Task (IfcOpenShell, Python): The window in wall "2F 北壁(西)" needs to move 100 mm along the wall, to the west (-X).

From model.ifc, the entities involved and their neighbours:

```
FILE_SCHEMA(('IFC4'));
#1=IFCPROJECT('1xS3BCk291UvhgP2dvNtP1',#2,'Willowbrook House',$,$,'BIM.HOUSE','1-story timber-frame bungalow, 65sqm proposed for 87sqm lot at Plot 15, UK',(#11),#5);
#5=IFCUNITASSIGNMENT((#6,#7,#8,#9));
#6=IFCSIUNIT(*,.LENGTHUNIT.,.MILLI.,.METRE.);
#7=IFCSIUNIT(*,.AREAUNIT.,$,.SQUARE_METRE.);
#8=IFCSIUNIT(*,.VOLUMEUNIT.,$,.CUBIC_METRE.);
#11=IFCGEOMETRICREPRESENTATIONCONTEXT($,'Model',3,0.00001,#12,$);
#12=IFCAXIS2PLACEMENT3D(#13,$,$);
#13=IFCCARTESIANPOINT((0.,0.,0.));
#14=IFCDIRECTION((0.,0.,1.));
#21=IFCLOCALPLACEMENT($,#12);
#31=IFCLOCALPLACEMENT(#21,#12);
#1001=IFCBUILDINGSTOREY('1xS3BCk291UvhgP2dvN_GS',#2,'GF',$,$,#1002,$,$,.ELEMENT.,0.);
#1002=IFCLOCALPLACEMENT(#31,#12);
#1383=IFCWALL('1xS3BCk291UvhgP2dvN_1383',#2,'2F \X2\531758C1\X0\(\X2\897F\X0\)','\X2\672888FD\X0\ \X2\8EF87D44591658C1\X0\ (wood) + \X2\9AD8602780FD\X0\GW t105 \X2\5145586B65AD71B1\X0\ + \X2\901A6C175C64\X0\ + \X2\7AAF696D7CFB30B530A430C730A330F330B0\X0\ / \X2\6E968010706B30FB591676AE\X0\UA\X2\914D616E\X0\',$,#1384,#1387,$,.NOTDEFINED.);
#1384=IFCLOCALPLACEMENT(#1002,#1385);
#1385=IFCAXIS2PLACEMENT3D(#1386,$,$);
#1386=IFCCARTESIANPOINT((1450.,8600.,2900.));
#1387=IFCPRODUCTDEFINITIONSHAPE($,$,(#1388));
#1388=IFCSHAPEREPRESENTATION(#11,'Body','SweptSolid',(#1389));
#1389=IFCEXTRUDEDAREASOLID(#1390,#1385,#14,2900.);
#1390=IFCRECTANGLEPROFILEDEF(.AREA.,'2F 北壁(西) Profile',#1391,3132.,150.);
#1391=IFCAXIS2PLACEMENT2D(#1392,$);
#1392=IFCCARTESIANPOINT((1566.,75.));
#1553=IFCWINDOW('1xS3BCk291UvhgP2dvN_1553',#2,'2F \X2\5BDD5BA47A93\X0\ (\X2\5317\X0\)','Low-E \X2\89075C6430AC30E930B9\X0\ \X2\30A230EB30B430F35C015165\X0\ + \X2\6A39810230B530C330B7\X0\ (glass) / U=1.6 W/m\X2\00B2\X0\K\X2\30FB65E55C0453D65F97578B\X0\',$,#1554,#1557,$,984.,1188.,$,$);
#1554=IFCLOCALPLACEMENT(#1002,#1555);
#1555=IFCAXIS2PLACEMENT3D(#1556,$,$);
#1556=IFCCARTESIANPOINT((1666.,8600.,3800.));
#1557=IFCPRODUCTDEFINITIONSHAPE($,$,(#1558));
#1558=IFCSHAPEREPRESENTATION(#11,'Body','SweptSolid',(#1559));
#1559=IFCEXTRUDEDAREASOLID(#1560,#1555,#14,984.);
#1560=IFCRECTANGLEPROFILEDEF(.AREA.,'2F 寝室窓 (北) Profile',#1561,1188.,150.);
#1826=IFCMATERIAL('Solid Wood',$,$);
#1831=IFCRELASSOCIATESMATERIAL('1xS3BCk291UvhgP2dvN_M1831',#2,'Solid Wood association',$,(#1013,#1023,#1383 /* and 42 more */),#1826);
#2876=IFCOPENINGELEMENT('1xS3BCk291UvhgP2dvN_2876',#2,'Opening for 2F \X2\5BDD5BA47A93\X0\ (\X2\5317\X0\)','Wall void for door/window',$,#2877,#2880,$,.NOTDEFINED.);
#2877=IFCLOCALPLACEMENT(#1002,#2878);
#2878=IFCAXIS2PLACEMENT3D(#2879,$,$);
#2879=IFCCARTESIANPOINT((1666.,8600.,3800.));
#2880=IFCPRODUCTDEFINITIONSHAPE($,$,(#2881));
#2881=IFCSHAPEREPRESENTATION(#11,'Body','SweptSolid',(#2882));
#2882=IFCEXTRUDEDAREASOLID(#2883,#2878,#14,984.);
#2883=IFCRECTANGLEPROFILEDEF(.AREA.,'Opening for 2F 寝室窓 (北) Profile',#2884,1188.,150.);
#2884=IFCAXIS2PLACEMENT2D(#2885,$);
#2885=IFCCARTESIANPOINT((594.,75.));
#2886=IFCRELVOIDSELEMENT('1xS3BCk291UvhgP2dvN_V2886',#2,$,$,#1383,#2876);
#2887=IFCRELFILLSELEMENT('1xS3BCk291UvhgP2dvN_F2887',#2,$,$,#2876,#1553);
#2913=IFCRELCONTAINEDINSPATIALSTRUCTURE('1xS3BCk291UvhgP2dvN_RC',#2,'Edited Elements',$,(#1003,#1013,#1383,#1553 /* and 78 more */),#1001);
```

```python
import ifcopenshell
import ifcopenshell.api.geometry
import ifcopenshell.util.placement

model = ifcopenshell.open("model.ifc")

window = model.by_guid("1xS3BCk291UvhgP2dvN_1553")
opening = window.FillsVoids[0].RelatingOpeningElement
wall = opening.VoidsElements[0].RelatingBuildingElement

wall_matrix = ifcopenshell.util.placement.get_local_placement(wall.ObjectPlacement)
shift = wall_matrix[:3, 0] * -100.0
before = ifcopenshell.util.placement.get_local_placement(window.ObjectPlacement)[:3, 3].copy()

# The window is not placed relative to its opening, so move both.
for product in (opening, window):
    matrix = ifcopenshell.util.placement.get_local_placement(product.ObjectPlacement)
    matrix[:3, 3] += shift
    ifcopenshell.api.geometry.edit_object_placement(model, product=product, matrix=matrix, is_si=False)

after = ifcopenshell.util.placement.get_local_placement(window.ObjectPlacement)[:3, 3]
print("window moved by", (after - before).round(3) + 0.0)

model.write("model_v2.ifc")
```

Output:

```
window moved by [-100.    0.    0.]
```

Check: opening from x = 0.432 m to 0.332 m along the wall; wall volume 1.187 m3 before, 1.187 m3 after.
